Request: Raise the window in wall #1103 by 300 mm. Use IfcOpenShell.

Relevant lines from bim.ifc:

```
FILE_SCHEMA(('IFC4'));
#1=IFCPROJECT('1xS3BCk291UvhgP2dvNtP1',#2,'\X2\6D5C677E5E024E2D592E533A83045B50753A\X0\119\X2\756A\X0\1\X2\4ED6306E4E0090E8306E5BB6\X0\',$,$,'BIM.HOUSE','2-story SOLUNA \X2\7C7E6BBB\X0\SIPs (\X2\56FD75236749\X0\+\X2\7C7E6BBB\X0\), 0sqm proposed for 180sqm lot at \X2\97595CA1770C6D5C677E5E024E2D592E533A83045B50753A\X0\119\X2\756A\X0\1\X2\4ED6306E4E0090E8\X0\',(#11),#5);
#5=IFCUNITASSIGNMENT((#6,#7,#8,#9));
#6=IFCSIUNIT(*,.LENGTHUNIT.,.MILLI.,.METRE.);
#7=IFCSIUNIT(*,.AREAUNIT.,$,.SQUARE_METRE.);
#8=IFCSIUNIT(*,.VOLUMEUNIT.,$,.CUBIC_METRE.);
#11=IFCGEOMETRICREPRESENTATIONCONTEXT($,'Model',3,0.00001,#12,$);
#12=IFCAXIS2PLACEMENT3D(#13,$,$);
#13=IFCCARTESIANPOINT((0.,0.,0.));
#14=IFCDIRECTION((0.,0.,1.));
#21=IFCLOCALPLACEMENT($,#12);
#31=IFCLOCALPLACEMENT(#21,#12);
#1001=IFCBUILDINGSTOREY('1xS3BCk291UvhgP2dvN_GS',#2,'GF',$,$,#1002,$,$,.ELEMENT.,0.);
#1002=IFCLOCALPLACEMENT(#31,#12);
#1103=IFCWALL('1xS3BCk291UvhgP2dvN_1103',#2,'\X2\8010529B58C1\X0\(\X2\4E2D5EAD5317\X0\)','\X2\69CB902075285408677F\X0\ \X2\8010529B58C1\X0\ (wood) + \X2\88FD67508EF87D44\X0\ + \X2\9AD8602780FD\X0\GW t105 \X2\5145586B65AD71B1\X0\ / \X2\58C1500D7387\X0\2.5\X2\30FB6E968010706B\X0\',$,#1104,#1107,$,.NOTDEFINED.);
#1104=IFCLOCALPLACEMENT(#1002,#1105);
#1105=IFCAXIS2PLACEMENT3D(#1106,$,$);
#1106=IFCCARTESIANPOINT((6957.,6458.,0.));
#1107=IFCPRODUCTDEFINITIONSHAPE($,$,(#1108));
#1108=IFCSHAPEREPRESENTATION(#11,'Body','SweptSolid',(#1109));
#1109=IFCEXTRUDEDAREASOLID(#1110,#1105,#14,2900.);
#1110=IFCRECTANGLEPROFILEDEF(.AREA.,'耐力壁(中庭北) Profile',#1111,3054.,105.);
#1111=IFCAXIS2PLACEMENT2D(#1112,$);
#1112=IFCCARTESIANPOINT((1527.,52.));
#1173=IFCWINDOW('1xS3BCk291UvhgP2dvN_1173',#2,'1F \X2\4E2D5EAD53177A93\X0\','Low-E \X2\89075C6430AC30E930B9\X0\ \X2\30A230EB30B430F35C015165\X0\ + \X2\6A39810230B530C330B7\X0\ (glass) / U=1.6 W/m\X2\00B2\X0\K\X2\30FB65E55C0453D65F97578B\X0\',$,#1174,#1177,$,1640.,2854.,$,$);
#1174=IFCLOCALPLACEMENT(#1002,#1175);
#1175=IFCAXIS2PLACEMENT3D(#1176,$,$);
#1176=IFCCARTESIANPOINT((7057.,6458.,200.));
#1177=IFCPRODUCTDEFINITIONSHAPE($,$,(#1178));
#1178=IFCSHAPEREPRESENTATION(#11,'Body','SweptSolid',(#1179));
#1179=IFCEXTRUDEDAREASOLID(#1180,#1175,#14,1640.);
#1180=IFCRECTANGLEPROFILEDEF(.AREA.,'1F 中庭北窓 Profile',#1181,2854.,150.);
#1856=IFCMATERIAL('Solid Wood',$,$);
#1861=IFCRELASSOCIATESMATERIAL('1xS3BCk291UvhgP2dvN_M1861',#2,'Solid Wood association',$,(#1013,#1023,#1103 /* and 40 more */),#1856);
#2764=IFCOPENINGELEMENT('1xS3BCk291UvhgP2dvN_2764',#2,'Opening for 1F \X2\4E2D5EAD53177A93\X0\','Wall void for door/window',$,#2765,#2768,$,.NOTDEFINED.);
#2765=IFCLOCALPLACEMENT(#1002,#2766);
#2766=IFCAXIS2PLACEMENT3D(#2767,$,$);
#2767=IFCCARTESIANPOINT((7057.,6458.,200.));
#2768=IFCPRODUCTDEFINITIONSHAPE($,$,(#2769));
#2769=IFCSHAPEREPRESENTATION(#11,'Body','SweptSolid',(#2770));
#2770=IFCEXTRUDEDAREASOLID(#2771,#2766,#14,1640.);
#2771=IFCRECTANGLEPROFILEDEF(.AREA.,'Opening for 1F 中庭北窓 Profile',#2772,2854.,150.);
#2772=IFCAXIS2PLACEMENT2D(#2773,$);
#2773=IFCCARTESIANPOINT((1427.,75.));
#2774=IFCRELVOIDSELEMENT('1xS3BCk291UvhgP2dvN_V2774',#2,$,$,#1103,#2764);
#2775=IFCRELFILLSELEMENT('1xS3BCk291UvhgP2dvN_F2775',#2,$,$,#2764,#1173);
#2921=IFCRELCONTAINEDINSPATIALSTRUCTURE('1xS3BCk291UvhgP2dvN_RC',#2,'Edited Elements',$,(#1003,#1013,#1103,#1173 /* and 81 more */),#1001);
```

```python
import numpy as np
import ifcopenshell
import ifcopenshell.api.geometry
import ifcopenshell.util.placement
import ifcopenshell.util.unit

model = ifcopenshell.open("bim.ifc")
unit_scale = ifcopenshell.util.unit.calculate_unit_scale(model)

window = model.by_id(1173)
opening = window.FillsVoids[0].RelatingOpeningElement
dz = 0.3 / unit_scale

shift = np.array([0.0, 0.0, dz])
# The window is not placed relative to its opening, so move both.
for product in (opening, window):
    matrix = ifcopenshell.util.placement.get_local_placement(product.ObjectPlacement)
    matrix[:3, 3] += shift
    ifcopenshell.api.geometry.edit_object_placement(model, product=product, matrix=matrix, is_si=False)

print(f"moved by {dz * unit_scale:+.3f} m")

model.write("bim_edited.ifc")
```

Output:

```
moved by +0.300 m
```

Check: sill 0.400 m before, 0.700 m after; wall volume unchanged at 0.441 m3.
